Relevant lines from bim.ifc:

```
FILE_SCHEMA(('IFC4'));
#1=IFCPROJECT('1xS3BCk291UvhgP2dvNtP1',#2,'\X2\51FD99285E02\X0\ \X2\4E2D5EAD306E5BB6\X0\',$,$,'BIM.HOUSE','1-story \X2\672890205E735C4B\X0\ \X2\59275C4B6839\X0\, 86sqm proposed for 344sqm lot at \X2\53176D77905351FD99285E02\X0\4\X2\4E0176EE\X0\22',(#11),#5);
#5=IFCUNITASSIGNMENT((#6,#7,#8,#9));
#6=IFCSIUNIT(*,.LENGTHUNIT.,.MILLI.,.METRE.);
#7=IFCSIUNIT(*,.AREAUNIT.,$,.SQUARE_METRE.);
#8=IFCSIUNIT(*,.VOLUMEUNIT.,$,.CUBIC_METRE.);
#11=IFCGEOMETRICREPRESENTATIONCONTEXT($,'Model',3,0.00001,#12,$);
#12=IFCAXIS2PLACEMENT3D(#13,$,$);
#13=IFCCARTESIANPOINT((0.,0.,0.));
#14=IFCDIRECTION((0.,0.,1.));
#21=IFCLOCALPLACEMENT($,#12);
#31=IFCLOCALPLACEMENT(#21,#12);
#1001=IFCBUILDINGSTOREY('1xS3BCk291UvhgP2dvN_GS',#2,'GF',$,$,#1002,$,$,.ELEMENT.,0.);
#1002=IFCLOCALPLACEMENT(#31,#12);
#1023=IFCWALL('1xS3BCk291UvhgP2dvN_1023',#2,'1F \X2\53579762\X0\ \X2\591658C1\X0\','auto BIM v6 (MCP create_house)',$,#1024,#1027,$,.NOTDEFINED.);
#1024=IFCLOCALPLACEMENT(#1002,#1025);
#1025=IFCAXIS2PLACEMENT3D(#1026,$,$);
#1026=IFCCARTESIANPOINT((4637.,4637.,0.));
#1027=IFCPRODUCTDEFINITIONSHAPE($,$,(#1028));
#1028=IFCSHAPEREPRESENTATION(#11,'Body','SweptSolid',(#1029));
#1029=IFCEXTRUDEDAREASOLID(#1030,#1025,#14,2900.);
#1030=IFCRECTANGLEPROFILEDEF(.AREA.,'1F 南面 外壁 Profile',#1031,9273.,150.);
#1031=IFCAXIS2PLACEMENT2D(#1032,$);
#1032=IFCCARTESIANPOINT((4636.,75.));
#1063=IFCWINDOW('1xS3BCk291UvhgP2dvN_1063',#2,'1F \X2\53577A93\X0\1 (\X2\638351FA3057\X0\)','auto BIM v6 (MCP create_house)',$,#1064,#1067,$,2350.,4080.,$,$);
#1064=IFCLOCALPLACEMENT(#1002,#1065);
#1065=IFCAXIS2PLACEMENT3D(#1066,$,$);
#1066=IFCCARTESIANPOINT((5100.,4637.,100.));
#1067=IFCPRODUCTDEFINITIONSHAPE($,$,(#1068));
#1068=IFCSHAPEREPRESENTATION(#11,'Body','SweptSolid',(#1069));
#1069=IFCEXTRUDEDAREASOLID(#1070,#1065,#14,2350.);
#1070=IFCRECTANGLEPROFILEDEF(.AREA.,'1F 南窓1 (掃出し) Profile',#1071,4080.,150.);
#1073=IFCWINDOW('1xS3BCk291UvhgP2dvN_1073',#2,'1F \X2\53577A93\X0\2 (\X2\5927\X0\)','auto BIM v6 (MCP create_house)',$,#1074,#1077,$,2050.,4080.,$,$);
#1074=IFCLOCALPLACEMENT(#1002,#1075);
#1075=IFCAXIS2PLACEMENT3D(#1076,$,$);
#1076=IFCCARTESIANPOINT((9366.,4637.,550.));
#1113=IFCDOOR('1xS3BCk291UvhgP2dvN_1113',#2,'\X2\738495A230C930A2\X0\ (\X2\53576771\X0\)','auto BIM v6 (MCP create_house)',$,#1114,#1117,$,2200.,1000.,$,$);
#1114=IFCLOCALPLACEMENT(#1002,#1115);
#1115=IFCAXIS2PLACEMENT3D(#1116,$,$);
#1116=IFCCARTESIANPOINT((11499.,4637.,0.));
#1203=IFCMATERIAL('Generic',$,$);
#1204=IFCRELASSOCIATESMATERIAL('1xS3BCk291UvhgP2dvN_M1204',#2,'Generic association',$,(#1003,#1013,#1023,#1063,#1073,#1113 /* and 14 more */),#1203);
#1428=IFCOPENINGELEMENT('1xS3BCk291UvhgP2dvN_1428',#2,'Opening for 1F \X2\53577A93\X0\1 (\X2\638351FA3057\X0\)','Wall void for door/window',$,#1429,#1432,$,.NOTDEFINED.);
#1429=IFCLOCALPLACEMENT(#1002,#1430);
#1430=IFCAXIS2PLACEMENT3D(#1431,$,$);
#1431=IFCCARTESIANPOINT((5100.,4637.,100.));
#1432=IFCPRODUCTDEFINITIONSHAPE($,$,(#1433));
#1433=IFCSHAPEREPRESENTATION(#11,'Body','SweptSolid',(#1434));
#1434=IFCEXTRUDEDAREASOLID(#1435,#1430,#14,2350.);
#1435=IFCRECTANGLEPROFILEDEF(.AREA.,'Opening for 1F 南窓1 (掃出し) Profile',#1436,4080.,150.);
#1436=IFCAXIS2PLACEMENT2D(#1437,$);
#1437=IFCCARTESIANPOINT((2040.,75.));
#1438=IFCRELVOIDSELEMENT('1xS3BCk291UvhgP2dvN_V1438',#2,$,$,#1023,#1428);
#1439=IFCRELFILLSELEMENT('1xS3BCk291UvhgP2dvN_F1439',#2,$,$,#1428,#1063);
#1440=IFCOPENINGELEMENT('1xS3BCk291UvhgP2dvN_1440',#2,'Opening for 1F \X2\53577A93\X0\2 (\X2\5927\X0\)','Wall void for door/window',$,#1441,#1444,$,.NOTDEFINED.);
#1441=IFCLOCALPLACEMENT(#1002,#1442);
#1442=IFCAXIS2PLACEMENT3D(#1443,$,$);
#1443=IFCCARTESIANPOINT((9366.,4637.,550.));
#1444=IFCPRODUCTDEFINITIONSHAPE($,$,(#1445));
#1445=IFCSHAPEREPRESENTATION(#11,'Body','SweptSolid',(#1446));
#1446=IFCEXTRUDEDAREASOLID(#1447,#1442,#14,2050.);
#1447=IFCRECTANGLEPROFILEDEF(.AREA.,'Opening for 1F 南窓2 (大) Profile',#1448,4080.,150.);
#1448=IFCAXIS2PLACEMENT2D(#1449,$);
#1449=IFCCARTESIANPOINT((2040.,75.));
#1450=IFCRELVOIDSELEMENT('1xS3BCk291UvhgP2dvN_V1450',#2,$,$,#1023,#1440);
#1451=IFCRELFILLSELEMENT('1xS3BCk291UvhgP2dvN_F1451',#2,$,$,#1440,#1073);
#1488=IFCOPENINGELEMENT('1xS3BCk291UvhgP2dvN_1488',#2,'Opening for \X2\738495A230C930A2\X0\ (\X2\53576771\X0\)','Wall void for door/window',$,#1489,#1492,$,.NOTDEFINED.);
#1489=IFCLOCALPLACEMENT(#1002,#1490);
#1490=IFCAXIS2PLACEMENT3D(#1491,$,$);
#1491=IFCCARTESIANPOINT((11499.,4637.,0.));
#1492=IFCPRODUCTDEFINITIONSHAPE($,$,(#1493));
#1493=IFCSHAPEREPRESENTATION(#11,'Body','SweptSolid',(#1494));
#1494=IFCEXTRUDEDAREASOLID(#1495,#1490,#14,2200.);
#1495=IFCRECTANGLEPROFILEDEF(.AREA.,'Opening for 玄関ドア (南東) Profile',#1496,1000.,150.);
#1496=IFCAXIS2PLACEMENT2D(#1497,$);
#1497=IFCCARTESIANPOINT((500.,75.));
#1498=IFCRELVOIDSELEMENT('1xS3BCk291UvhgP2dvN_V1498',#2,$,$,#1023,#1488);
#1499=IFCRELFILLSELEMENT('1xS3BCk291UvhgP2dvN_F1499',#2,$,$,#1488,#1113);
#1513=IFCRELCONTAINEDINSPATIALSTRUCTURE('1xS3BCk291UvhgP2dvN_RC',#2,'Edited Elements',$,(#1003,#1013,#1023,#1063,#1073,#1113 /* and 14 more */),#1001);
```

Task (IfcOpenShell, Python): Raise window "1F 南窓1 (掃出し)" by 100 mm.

```python
import numpy as np
import ifcopenshell
import ifcopenshell.api.geometry
import ifcopenshell.util.placement
import ifcopenshell.util.unit

model = ifcopenshell.open("bim.ifc")
unit_scale = ifcopenshell.util.unit.calculate_unit_scale(model)

window = model.by_id(1063)
opening = window.FillsVoids[0].RelatingOpeningElement
dz = 100.0

shift = np.array([0.0, 0.0, dz])
# The window is not placed relative to its opening, so move both.
for product in (opening, window):
    matrix = ifcopenshell.util.placement.get_local_placement(product.ObjectPlacement)
    matrix[:3, 3] += shift
    ifcopenshell.api.geometry.edit_object_placement(model, product=product, matrix=matrix, is_si=False)

print(f"moved by {dz * unit_scale:+.3f} m")

model.write("bim_rev.ifc")
```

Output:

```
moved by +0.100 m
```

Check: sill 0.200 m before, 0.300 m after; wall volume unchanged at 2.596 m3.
